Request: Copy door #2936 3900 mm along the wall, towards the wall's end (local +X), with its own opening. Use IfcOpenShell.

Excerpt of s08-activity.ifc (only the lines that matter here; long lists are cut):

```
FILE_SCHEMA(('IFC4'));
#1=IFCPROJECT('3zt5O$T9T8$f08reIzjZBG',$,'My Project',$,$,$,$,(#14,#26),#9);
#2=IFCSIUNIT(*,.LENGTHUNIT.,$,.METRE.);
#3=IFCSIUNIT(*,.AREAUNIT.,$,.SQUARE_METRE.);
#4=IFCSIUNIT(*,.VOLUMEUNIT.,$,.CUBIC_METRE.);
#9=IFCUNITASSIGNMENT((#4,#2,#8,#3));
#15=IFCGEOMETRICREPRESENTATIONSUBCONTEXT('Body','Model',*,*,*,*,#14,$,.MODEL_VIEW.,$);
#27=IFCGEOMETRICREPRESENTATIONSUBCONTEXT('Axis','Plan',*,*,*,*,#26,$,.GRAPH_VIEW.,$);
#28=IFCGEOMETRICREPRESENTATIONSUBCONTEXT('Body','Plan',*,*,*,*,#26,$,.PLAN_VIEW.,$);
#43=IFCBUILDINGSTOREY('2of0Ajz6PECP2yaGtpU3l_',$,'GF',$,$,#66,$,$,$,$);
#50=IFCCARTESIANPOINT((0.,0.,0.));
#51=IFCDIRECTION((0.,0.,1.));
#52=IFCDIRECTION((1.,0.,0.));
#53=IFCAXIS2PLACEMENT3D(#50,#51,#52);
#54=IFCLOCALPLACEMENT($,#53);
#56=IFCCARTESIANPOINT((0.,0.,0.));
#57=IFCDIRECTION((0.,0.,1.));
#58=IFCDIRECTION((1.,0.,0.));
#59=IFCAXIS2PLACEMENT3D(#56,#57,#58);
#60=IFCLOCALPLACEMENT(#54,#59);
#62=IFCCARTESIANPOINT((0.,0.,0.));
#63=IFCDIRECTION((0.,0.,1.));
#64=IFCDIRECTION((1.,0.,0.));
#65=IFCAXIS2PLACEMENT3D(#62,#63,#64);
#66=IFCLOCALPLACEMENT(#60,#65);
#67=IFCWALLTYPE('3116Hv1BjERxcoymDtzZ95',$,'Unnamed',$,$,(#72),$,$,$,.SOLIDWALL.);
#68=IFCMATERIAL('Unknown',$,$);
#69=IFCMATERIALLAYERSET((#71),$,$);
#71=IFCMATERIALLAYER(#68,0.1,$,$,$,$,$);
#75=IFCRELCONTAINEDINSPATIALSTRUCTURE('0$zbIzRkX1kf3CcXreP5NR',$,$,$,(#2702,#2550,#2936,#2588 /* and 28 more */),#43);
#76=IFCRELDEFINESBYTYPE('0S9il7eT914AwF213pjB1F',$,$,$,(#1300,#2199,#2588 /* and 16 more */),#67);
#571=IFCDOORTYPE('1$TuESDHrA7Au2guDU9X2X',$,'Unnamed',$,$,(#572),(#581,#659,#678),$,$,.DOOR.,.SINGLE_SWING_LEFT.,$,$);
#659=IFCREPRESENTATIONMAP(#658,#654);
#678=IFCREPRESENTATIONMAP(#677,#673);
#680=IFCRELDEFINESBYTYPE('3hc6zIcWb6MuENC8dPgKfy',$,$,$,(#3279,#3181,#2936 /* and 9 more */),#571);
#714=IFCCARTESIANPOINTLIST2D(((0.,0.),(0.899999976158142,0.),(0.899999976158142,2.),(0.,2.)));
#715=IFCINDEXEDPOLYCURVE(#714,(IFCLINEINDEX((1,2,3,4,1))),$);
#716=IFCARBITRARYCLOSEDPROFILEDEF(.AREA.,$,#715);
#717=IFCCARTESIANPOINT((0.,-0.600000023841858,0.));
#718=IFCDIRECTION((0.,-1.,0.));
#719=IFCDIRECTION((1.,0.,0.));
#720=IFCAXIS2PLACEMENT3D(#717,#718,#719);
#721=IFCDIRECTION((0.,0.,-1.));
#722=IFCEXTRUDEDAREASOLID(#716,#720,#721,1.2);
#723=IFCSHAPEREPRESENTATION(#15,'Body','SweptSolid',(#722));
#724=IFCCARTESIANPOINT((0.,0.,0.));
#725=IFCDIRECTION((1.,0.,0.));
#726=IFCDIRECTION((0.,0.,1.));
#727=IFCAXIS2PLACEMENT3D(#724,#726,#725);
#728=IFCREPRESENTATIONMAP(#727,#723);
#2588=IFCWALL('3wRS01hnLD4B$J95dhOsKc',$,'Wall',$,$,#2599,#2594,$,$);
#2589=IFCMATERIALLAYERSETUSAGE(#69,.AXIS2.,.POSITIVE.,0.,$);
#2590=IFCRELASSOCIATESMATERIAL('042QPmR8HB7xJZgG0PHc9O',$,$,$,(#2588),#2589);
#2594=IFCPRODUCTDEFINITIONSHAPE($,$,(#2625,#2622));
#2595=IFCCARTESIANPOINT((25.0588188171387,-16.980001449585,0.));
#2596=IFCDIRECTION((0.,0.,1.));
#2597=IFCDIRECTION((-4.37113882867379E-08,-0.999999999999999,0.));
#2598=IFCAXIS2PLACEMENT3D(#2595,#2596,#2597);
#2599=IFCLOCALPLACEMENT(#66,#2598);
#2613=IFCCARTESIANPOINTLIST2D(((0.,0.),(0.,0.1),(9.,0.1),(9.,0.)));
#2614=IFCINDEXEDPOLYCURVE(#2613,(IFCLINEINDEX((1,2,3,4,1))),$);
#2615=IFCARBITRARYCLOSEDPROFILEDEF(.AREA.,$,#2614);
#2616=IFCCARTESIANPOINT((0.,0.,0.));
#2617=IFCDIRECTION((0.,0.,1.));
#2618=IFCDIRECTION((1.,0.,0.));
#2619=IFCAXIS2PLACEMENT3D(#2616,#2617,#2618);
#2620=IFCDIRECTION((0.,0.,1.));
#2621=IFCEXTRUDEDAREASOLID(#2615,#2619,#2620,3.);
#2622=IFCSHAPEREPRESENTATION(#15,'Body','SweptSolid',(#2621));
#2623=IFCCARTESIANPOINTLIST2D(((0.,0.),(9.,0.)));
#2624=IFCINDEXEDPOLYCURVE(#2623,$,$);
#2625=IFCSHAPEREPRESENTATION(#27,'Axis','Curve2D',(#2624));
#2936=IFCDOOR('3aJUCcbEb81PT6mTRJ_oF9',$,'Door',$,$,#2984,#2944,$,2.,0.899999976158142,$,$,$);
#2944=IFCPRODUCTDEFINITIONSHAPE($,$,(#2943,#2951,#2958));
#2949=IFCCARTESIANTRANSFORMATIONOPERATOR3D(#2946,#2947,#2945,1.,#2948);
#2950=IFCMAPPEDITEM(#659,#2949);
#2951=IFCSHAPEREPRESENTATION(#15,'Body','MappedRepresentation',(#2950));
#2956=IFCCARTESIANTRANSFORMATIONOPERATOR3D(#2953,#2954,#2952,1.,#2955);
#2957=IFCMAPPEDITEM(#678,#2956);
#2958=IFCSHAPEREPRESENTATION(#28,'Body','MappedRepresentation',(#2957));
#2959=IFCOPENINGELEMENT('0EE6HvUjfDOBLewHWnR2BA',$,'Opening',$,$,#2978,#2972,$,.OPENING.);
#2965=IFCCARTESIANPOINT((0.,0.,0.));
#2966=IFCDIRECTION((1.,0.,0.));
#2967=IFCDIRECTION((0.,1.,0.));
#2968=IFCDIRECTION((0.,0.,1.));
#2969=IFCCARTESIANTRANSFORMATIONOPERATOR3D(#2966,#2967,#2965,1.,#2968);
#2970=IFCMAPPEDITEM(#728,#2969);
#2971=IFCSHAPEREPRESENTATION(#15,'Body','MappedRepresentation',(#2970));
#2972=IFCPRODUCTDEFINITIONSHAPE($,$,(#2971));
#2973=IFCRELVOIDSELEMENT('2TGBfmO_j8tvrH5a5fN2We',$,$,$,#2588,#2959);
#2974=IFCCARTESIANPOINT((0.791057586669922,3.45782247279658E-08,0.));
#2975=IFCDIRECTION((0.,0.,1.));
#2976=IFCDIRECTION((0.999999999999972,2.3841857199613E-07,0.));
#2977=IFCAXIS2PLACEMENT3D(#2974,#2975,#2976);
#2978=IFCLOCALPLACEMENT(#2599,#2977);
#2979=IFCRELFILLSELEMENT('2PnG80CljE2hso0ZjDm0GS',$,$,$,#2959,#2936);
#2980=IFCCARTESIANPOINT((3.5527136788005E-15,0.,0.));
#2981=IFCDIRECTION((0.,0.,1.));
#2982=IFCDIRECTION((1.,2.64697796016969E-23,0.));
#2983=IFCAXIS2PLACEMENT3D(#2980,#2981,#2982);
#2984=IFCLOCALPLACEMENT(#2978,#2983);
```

```python
import ifcopenshell
import ifcopenshell.api.feature
import ifcopenshell.api.geometry
import ifcopenshell.api.root
import ifcopenshell.geom
import ifcopenshell.util.element
import ifcopenshell.util.placement
import ifcopenshell.util.shape

model = ifcopenshell.open("s08-activity.ifc")
settings = ifcopenshell.geom.settings()


def volume(element):
    """Net volume in cubic metres, openings subtracted."""
    shape = ifcopenshell.geom.create_shape(settings, element)
    return ifcopenshell.util.shape.get_volume(shape.geometry)


door = model.by_guid("3aJUCcbEb81PT6mTRJ_oF9")
opening = door.FillsVoids[0].RelatingOpeningElement
wall = opening.VoidsElements[0].RelatingBuildingElement
before = volume(wall)
shift = ifcopenshell.util.placement.get_local_placement(wall.ObjectPlacement)[:3, 0] * 3.9

# copy_class copies the void relationship, type, container and properties, but no geometry.
new_opening = ifcopenshell.api.root.copy_class(model, product=opening)
new_opening.Representation = ifcopenshell.util.element.copy_deep(
    model, opening.Representation, exclude=["IfcGeometricRepresentationContext", "IfcRepresentationMap"]
)
new_door = ifcopenshell.api.root.copy_class(model, product=door)
new_door.Representation = ifcopenshell.util.element.copy_deep(
    model, door.Representation, exclude=["IfcGeometricRepresentationContext", "IfcRepresentationMap"]
)
ifcopenshell.api.feature.add_filling(model, opening=new_opening, element=new_door)

for old, new in ((opening, new_opening), (door, new_door)):
    matrix = ifcopenshell.util.placement.get_local_placement(old.ObjectPlacement)
    matrix[:3, 3] += shift
    ifcopenshell.api.geometry.edit_object_placement(model, product=new, matrix=matrix, is_si=False)

after = volume(wall)

print(f"wall volume {before:.3f} -> {after:.3f} m3")

model.write("s08-activity_edited.ifc")
```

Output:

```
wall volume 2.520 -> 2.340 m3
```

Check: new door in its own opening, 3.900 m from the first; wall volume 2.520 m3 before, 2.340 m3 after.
